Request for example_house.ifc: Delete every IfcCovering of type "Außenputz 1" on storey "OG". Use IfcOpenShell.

First a look at what the model holds.

```python
import ifcopenshell
import ifcopenshell.util.element

model = ifcopenshell.open("example_house.ifc")
print(model.schema)
storey = next(s for s in model.by_type("IfcBuildingStorey") if s.Name == "OG")
coverings = [e for e in ifcopenshell.util.element.get_decomposition(storey) if e.is_a("IfcCovering")]
seen = {}
for e in coverings:
    element_type = ifcopenshell.util.element.get_type(e)
    name = element_type.Name if element_type not in (None, e) else None
    seen[name] = seen.get(name, 0) + 1
for name, count in sorted(seen.items(), key=str):
    print(count, "x", name)
```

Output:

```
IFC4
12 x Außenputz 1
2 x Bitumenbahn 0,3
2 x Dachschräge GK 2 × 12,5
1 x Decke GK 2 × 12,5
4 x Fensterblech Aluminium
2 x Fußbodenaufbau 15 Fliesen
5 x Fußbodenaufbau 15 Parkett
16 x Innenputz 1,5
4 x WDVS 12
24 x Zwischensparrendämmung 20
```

```python
import ifcopenshell
import ifcopenshell.api.root
import ifcopenshell.util.element

model = ifcopenshell.open("example_house.ifc")

storey = next(s for s in model.by_type("IfcBuildingStorey") if s.Name == "OG")
coverings = [e for e in ifcopenshell.util.element.get_decomposition(storey) if e.is_a("IfcCovering")]
targets = [e for e in coverings if (t := ifcopenshell.util.element.get_type(e)) not in (None, e) and t.Name == "Außenputz 1"]

for e in targets:
    ifcopenshell.api.root.remove_product(model, product=e)
print(len(targets), "removed")

model.write("example_house_v2.ifc")
```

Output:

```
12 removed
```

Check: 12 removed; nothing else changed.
